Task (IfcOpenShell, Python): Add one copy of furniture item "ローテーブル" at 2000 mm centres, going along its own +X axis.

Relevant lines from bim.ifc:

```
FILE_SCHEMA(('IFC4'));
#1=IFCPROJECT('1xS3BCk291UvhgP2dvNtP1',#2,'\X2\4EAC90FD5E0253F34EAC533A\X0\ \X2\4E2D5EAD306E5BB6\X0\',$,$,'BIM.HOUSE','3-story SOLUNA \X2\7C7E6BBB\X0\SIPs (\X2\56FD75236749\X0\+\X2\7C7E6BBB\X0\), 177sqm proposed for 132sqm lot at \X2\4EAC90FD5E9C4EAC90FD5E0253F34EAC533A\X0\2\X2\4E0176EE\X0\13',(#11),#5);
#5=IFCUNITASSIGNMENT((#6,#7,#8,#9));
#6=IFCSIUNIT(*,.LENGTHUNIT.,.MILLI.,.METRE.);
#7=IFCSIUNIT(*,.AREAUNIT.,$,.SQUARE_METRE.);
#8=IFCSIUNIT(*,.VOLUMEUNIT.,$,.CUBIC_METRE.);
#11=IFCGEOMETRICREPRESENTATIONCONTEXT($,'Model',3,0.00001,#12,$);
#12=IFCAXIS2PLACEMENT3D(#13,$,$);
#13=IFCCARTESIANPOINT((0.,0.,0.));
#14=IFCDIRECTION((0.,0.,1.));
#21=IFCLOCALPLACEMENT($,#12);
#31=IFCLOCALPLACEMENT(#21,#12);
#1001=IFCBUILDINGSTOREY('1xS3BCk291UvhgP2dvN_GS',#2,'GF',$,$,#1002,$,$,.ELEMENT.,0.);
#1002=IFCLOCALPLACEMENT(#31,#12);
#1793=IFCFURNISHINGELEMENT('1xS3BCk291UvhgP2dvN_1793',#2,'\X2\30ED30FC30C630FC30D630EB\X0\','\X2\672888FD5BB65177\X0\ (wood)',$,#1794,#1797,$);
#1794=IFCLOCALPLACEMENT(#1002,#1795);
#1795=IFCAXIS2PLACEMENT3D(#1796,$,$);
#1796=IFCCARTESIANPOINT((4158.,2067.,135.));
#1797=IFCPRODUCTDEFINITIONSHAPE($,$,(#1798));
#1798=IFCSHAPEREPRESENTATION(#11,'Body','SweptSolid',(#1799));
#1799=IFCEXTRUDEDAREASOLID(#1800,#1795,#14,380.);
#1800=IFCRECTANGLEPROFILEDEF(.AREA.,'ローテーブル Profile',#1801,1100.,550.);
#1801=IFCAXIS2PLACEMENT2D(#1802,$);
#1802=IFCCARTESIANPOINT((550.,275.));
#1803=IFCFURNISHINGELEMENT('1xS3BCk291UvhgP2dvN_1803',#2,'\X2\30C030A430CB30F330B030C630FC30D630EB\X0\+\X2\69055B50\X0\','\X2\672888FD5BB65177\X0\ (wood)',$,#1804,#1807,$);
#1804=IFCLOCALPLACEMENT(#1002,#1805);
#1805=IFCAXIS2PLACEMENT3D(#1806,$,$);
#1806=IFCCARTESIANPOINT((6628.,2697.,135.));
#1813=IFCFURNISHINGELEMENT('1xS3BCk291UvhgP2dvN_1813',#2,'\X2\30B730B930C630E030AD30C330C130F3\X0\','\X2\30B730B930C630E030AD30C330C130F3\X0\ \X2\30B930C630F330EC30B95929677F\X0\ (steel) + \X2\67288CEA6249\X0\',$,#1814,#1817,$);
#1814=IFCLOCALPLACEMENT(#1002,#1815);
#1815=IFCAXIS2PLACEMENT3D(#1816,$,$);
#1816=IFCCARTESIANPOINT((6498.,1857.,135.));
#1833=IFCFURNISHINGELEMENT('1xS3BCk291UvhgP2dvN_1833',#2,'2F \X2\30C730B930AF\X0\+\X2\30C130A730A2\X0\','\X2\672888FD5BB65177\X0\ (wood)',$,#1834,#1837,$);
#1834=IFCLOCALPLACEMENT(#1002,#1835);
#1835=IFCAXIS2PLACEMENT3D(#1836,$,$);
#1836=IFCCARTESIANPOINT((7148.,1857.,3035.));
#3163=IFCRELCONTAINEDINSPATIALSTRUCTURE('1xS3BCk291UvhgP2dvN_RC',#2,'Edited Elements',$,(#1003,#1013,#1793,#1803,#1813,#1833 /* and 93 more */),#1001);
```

```python
import ifcopenshell
import ifcopenshell.api.geometry
import ifcopenshell.api.root
import ifcopenshell.util.element
import ifcopenshell.util.placement

model = ifcopenshell.open("bim.ifc")


def reuse_history(source, copy):
    """copy_class also copies each property set's owner history, people and application; keep the originals."""
    for rel in copy.IsDefinedBy:
        if rel.is_a("IfcRelDefinesByProperties") and (history := rel.RelatingPropertyDefinition.OwnerHistory):
            rel.RelatingPropertyDefinition.OwnerHistory = source.OwnerHistory
            ifcopenshell.util.element.remove_deep2(model, history)


source = model.by_guid("1xS3BCk291UvhgP2dvN_1793")
base = ifcopenshell.util.placement.get_local_placement(source.ObjectPlacement)
step = base[:3, 0] * 2000.0

for i in range(1, 2):
    copy = ifcopenshell.api.root.copy_class(model, product=source)
    copy.Representation = ifcopenshell.util.element.copy_deep(
        model, source.Representation, exclude=["IfcGeometricRepresentationContext", "IfcRepresentationMap"]
    )
    reuse_history(source, copy)
    matrix = base.copy()
    matrix[:3, 3] += i * step
    print("added at", matrix[:3, 3].round(3) + 0.0)
    ifcopenshell.api.geometry.edit_object_placement(model, product=copy, matrix=matrix, is_si=False)

model.write("bim_updated.ifc")
```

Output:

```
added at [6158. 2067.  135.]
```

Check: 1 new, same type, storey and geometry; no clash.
